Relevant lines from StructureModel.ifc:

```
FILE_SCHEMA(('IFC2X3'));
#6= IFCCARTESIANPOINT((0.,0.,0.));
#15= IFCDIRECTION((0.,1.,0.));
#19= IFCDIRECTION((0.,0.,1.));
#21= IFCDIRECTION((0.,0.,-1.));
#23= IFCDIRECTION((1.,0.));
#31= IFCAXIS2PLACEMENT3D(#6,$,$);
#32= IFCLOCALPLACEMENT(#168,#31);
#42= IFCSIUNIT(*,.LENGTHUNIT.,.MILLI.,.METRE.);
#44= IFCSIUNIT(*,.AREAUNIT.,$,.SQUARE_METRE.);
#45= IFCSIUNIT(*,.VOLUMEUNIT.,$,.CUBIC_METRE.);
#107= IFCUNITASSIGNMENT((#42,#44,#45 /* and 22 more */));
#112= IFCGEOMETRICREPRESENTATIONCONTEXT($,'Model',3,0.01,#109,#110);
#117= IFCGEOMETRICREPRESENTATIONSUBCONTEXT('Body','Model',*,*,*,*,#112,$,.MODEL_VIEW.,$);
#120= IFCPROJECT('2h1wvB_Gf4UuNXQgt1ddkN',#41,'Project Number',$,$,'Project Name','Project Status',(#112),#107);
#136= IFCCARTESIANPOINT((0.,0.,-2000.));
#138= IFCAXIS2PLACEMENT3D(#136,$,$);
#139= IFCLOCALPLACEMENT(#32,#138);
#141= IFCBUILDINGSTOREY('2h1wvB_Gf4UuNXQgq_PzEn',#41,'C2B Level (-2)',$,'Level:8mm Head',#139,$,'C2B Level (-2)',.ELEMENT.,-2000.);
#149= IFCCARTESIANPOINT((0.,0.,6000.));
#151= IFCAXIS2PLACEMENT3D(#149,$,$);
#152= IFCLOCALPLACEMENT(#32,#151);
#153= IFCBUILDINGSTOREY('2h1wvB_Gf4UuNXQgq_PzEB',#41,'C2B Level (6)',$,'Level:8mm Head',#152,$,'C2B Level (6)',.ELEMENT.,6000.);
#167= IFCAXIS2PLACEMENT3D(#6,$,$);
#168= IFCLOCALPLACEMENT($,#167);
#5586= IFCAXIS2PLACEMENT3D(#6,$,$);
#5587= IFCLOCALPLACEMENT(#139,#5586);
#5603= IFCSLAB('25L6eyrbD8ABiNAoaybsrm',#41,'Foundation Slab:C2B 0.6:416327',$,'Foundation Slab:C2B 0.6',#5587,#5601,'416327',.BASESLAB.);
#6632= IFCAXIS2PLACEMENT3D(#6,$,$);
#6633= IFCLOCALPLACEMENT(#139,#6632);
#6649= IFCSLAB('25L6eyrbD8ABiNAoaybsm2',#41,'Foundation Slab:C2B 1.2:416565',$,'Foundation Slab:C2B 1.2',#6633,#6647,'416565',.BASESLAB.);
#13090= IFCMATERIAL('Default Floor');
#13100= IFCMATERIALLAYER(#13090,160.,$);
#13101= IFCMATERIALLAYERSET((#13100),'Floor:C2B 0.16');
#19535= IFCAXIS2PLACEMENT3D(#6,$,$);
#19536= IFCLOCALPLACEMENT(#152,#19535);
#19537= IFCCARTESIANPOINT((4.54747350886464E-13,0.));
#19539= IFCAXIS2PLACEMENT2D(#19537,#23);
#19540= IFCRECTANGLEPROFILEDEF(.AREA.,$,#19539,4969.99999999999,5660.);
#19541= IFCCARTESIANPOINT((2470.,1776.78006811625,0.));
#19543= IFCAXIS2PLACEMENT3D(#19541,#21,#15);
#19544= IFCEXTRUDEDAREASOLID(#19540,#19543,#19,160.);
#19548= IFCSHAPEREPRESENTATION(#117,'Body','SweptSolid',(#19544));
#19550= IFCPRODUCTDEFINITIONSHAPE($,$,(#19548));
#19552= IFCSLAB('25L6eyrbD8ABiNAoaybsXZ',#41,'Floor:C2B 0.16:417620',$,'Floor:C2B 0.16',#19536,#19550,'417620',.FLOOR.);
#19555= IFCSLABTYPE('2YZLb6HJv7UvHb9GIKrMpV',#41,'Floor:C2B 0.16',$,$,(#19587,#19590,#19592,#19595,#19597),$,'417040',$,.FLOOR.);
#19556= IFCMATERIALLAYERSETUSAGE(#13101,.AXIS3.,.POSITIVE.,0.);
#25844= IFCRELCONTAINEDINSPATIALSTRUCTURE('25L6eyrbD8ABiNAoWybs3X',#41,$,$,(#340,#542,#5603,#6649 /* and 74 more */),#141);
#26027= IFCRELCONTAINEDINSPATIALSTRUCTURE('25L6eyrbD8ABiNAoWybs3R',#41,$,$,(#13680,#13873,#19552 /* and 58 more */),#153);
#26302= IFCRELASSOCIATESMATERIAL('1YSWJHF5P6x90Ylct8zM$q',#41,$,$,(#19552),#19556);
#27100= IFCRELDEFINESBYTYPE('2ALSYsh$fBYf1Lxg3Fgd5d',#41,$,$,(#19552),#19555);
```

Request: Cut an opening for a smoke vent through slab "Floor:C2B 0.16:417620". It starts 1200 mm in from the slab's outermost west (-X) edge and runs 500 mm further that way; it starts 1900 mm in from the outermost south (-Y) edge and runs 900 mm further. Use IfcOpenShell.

```python
import numpy as np
import ifcopenshell
import ifcopenshell.api.feature
import ifcopenshell.api.geometry
import ifcopenshell.api.root
import ifcopenshell.geom
import ifcopenshell.util.placement
import ifcopenshell.util.representation
import ifcopenshell.util.shape
import ifcopenshell.util.unit

model = ifcopenshell.open("StructureModel.ifc")
unit_scale = ifcopenshell.util.unit.calculate_unit_scale(model)
settings = ifcopenshell.geom.settings()


def volume(element):
    """Net volume in cubic metres, openings subtracted."""
    shape = ifcopenshell.geom.create_shape(settings, element)
    return ifcopenshell.util.shape.get_volume(shape.geometry)


slab = model.by_guid("25L6eyrbD8ABiNAoaybsXZ")
before = volume(slab)

# Extent in the slab's own axes, in metres. The edges named are its -X and -Y sides.
slab_shape = ifcopenshell.geom.create_shape(settings, slab)
vertices = ifcopenshell.util.shape.get_vertices(slab_shape.geometry)
x_min, y_min, bottom = vertices.min(axis=0)
top = vertices[:, 2].max()

opening = ifcopenshell.api.root.create_entity(model, ifc_class="IfcOpeningElement", name="Smoke vent opening")
context = ifcopenshell.util.representation.get_context(model, "Model", "Body", "MODEL_VIEW")
width, depth = 0.5, 0.9
outline = [(0.0, 0.0), (width, 0.0), (width, depth), (0.0, depth), (0.0, 0.0)]
# Overshoot both faces by 50 mm so the cut is clean.
shape = ifcopenshell.api.geometry.add_slab_representation(
    model, context=context, depth=top - bottom + 0.1, polyline=outline
)
ifcopenshell.api.geometry.assign_representation(model, product=opening, representation=shape)

matrix = ifcopenshell.util.placement.get_local_placement(slab.ObjectPlacement)
matrix[:, 3] = matrix @ np.append(np.array([x_min + 1.2, y_min + 1.9, bottom - 0.05]) / unit_scale, 1.0)
ifcopenshell.api.geometry.edit_object_placement(model, product=opening, matrix=matrix, is_si=False)
ifcopenshell.api.feature.add_feature(model, feature=opening, element=slab)

after = volume(slab)

print(f"slab volume {before:.3f} -> {after:.3f} m3")

model.write("StructureModel_edited.ifc")
```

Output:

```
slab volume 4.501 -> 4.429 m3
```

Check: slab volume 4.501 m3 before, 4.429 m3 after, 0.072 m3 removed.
